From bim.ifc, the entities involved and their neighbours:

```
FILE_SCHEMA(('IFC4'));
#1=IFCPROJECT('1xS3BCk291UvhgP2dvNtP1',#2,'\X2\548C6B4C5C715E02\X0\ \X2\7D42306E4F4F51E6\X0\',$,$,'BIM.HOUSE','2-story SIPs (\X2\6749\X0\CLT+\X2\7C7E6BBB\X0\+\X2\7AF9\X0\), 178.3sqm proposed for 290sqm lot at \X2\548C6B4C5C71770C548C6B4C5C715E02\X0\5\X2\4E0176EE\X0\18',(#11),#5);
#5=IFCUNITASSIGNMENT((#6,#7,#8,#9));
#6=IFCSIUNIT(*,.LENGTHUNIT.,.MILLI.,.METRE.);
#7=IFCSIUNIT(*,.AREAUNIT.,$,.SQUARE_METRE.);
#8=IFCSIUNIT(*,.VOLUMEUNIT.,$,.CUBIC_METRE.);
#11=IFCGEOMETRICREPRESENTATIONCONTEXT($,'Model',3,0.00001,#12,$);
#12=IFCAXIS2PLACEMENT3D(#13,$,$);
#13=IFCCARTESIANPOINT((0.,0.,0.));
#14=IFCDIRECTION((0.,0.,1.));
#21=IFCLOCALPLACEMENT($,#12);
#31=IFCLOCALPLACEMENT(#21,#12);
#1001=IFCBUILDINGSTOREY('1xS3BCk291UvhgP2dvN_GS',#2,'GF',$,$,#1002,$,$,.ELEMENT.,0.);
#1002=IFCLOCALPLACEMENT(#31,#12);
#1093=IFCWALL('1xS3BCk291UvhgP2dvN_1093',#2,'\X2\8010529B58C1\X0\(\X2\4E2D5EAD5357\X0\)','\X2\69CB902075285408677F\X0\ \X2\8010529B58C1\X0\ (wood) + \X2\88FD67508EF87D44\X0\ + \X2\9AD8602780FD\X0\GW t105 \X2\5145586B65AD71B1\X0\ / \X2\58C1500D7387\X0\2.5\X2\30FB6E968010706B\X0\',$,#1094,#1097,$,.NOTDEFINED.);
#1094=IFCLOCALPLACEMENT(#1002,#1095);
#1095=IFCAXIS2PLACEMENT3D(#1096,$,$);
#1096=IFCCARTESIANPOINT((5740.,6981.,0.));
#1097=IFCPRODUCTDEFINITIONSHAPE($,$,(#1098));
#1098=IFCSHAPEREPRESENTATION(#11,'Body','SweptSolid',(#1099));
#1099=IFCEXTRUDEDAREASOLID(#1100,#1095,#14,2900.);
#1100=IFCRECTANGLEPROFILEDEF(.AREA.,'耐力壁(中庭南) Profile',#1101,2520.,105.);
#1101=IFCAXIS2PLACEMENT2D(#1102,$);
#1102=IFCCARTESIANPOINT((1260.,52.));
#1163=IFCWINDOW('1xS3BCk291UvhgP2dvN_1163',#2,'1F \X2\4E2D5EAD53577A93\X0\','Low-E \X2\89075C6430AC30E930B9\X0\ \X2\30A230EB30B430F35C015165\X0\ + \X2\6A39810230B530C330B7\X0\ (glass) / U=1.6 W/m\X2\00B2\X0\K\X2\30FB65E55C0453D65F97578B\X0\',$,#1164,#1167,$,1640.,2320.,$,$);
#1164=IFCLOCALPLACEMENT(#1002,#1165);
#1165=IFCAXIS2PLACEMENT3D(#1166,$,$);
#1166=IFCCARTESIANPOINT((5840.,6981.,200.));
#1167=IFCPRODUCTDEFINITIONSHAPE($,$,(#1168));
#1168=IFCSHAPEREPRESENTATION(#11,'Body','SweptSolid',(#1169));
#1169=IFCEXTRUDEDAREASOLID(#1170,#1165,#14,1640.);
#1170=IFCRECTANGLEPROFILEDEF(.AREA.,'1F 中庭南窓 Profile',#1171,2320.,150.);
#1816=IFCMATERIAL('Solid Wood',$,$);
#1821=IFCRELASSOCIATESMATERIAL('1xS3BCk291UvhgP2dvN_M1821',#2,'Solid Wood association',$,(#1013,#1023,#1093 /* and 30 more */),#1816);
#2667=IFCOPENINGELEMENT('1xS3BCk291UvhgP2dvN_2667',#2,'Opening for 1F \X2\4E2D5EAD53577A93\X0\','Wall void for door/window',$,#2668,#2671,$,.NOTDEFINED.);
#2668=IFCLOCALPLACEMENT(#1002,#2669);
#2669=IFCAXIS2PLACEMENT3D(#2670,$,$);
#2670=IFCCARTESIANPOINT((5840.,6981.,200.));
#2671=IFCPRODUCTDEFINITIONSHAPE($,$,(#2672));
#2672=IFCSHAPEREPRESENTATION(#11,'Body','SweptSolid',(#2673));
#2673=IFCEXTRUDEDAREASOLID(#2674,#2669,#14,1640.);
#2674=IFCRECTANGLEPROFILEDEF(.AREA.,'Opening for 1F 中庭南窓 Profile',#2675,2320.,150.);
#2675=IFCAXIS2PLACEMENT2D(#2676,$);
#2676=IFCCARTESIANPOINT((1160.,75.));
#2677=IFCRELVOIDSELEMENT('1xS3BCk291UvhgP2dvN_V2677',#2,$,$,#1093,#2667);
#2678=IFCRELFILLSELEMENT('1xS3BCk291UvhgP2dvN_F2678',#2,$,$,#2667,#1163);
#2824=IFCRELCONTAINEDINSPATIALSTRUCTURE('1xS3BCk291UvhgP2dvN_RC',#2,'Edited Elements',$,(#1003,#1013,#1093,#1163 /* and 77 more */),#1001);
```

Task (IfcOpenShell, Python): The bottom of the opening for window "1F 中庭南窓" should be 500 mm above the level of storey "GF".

```python
import numpy as np
import ifcopenshell
import ifcopenshell.api.geometry
import ifcopenshell.geom
import ifcopenshell.util.element
import ifcopenshell.util.placement
import ifcopenshell.util.shape
import ifcopenshell.util.unit

model = ifcopenshell.open("bim.ifc")
unit_scale = ifcopenshell.util.unit.calculate_unit_scale(model)

window = model.by_id(1163)
opening = window.FillsVoids[0].RelatingOpeningElement
storey = ifcopenshell.util.element.get_container(window, ifc_class="IfcBuildingStorey")
level = ifcopenshell.util.placement.get_local_placement(storey.ObjectPlacement)[2, 3]

# The opening's origin need not be at the sill, so measure its lowest point.
shape = ifcopenshell.geom.create_shape(ifcopenshell.geom.settings(), opening)
bottom = ifcopenshell.util.shape.get_shape_bottom_elevation(shape, shape.geometry) / unit_scale
dz = level + 0.5 / unit_scale - bottom

shift = np.array([0.0, 0.0, dz])
# The window is not placed relative to its opening, so move both.
for product in (opening, window):
    matrix = ifcopenshell.util.placement.get_local_placement(product.ObjectPlacement)
    matrix[:3, 3] += shift
    ifcopenshell.api.geometry.edit_object_placement(model, product=product, matrix=matrix, is_si=False)

print(f"moved by {dz * unit_scale:+.3f} m")

model.write("bim_updated.ifc")
```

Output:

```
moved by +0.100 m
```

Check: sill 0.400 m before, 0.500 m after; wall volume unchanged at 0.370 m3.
